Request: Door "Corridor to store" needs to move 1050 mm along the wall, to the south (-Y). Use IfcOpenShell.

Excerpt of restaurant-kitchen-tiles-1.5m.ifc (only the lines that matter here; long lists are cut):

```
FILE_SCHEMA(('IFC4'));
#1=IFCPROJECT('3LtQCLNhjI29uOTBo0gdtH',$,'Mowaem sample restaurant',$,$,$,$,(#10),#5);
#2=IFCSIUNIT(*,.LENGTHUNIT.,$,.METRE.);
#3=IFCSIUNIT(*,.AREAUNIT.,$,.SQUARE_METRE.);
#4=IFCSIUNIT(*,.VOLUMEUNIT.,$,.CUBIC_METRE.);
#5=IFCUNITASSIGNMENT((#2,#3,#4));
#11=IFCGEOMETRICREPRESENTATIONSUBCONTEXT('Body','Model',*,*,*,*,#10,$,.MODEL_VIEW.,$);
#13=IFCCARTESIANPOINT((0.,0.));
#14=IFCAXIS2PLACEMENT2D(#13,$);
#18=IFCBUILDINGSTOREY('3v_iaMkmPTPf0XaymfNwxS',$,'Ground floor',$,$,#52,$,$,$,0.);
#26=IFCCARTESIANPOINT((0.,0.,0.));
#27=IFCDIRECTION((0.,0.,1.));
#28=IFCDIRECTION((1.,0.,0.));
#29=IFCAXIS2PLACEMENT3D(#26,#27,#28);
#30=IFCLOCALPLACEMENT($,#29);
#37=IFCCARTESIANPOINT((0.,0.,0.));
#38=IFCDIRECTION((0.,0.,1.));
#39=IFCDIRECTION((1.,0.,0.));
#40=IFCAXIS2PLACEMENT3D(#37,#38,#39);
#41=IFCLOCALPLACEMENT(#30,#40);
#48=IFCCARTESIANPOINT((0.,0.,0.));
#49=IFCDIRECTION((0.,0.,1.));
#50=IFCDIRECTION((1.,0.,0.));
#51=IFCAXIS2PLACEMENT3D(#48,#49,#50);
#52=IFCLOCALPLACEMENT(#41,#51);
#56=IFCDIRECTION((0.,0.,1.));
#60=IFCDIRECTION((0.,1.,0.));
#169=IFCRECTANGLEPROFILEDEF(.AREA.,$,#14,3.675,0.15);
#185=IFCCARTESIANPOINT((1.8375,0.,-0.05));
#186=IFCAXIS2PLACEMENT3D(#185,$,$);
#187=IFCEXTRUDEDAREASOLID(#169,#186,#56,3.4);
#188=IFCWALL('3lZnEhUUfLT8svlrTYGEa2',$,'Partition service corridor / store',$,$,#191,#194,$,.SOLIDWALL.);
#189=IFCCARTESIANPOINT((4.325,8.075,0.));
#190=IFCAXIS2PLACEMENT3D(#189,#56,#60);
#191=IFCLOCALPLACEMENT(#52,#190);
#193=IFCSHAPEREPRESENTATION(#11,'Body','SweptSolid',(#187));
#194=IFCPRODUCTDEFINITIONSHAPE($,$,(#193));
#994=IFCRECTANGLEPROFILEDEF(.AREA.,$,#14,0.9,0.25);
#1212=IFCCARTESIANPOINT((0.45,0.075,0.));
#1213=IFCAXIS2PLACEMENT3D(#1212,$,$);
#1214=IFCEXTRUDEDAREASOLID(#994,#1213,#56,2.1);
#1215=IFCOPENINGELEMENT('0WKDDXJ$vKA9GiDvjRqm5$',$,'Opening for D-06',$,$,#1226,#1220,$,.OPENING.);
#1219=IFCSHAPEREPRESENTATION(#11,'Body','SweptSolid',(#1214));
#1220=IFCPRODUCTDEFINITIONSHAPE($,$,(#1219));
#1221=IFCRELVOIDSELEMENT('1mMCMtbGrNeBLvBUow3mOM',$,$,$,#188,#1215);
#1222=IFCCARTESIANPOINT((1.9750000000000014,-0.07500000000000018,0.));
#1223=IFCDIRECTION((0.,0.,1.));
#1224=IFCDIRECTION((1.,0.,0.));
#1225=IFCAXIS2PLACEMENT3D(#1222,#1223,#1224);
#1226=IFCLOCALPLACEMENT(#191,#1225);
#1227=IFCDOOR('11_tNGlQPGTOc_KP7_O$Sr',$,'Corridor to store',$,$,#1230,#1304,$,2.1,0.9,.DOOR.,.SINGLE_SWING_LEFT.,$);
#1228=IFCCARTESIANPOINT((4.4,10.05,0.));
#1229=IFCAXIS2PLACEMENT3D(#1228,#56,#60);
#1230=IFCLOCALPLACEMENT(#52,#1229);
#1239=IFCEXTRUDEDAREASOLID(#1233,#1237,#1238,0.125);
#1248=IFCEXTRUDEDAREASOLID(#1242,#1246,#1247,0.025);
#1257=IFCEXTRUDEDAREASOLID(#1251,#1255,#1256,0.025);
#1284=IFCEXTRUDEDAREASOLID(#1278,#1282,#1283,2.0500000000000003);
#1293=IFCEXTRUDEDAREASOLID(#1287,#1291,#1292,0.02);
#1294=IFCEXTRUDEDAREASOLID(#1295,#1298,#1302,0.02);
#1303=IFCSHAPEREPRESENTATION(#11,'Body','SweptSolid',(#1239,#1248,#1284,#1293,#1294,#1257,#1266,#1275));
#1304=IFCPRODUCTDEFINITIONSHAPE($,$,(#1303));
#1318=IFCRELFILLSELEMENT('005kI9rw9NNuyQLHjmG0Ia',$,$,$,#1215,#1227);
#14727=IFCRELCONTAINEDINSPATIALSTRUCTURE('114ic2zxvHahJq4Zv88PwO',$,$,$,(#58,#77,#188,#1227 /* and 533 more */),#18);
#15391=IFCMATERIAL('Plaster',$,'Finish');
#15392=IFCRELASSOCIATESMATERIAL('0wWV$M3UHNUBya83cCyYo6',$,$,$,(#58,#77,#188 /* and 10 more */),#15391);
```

```python
import ifcopenshell
import ifcopenshell.api.geometry
import ifcopenshell.util.placement

model = ifcopenshell.open("restaurant-kitchen-tiles-1.5m.ifc")

door = model.by_guid("11_tNGlQPGTOc_KP7_O$Sr")
opening = door.FillsVoids[0].RelatingOpeningElement
wall = opening.VoidsElements[0].RelatingBuildingElement

wall_matrix = ifcopenshell.util.placement.get_local_placement(wall.ObjectPlacement)
shift = wall_matrix[:3, 0] * -1.05
before = ifcopenshell.util.placement.get_local_placement(door.ObjectPlacement)[:3, 3].copy()

# The door is not placed relative to its opening, so move both.
for product in (opening, door):
    matrix = ifcopenshell.util.placement.get_local_placement(product.ObjectPlacement)
    matrix[:3, 3] += shift
    ifcopenshell.api.geometry.edit_object_placement(model, product=product, matrix=matrix, is_si=False)

after = ifcopenshell.util.placement.get_local_placement(door.ObjectPlacement)[:3, 3]
print("door moved by", (after - before).round(3) + 0.0)

model.write("restaurant-kitchen-tiles-1.5m-out.ifc")
```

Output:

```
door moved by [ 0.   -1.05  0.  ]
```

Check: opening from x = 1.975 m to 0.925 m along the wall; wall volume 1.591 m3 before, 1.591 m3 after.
